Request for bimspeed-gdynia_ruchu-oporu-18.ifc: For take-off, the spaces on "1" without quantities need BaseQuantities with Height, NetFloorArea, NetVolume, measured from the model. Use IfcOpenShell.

First a look at what the model holds.

```python
import ifcopenshell
import ifcopenshell.util.element
import ifcopenshell.util.unit

model = ifcopenshell.open("bimspeed-gdynia_ruchu-oporu-18.ifc")
print(model.schema)
for unit_type in ("LENGTHUNIT", "AREAUNIT", "VOLUMEUNIT"):
    print(unit_type, ifcopenshell.util.unit.calculate_unit_scale(model, unit_type))
storey = next(s for s in model.by_type("IfcBuildingStorey") if s.Name == "1")
spaces = [e for e in ifcopenshell.util.element.get_decomposition(storey) if e.is_a("IfcSpace")]
for e in sorted(spaces, key=lambda e: e.id()):
    print(e.id(), e.is_a(), e.Name, list(ifcopenshell.util.element.get_psets(e, qtos_only=True)), sep=" | ")
```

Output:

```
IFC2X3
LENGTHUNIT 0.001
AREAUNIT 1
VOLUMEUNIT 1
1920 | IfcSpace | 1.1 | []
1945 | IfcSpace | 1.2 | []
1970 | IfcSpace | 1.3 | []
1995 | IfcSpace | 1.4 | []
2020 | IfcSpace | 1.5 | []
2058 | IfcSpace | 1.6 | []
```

```python
import ifcopenshell
import ifcopenshell.api.pset
import ifcopenshell.geom
import ifcopenshell.util.element
import ifcopenshell.util.shape
import ifcopenshell.util.unit

model = ifcopenshell.open("bimspeed-gdynia_ruchu-oporu-18.ifc")
unit_scale = ifcopenshell.util.unit.calculate_unit_scale(model)
area_scale = ifcopenshell.util.unit.calculate_unit_scale(model, "AREAUNIT")
volume_scale = ifcopenshell.util.unit.calculate_unit_scale(model, "VOLUMEUNIT")
settings = ifcopenshell.geom.settings()

storey = next(s for s in model.by_type("IfcBuildingStorey") if s.Name == "1")
spaces = [e for e in ifcopenshell.util.element.get_decomposition(storey) if e.is_a("IfcSpace")]

for e in sorted(spaces, key=lambda e: e.id()):
    if ifcopenshell.util.element.get_psets(e, qtos_only=True, should_inherit=False):
        continue
    # Geometry comes back in metres, in the element's own axes.
    shape = ifcopenshell.geom.create_shape(settings, e)
    values = {
        "Height": ifcopenshell.util.shape.get_z(shape.geometry) / unit_scale,
        "NetFloorArea": ifcopenshell.util.shape.get_footprint_area(shape.geometry) / area_scale,
        "NetVolume": ifcopenshell.util.shape.get_volume(shape.geometry) / volume_scale,
    }
    qto = ifcopenshell.api.pset.add_qto(model, product=e, name="BaseQuantities")
    ifcopenshell.api.pset.edit_qto(model, qto=qto, properties=values)
    print(e.id(), {k: round(v, 3) for k, v in values.items()})

model.write("bimspeed-gdynia_ruchu-oporu-18_rev.ifc")
```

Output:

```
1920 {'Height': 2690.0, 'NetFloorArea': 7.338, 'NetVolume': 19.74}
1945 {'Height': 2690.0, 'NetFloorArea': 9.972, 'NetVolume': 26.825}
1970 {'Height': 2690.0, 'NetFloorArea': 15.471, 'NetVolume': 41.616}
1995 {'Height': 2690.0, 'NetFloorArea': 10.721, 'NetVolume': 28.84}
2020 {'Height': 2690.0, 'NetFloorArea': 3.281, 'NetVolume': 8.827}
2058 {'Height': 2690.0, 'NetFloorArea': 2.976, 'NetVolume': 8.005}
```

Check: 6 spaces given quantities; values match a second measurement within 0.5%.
